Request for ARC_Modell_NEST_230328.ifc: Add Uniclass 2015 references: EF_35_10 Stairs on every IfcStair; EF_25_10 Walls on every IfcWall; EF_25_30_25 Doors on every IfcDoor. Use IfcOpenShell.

First a look at what the model holds.

```python
import ifcopenshell

model = ifcopenshell.open("ARC_Modell_NEST_230328.ifc")
print(model.schema)
print("classifications:", [c.Name for c in model.by_type("IfcClassification")])
for ifc_class in ("IfcDoor", "IfcRoof", "IfcStair", "IfcWall", "IfcWindow"):
    print(ifc_class, len(model.by_type(ifc_class)))
```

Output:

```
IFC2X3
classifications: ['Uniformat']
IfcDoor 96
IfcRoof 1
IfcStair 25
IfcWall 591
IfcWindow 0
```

```python
import ifcopenshell
import ifcopenshell.api.classification

model = ifcopenshell.open("ARC_Modell_NEST_230328.ifc")

# IFC2X3 requires Source and Edition and has no link from the project to the system.
system = model.create_entity("IfcClassification", Source="NBS", Edition="2015", Name="Uniclass 2015")

codes = {
    "IfcStair": ("EF_35_10", "Stairs"),
    "IfcWall": ("EF_25_10", "Walls"),
    "IfcDoor": ("EF_25_30_25", "Doors"),
}
for ifc_class, (code, name) in codes.items():
    products = model.by_type(ifc_class)
    ifcopenshell.api.classification.add_reference(
        model, products=products, classification=system, identification=code, name=name
    )
    print(code, len(products))

model.write("ARC_Modell_NEST_230328_v2.ifc")
```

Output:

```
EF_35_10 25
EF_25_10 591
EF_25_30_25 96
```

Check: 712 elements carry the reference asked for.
